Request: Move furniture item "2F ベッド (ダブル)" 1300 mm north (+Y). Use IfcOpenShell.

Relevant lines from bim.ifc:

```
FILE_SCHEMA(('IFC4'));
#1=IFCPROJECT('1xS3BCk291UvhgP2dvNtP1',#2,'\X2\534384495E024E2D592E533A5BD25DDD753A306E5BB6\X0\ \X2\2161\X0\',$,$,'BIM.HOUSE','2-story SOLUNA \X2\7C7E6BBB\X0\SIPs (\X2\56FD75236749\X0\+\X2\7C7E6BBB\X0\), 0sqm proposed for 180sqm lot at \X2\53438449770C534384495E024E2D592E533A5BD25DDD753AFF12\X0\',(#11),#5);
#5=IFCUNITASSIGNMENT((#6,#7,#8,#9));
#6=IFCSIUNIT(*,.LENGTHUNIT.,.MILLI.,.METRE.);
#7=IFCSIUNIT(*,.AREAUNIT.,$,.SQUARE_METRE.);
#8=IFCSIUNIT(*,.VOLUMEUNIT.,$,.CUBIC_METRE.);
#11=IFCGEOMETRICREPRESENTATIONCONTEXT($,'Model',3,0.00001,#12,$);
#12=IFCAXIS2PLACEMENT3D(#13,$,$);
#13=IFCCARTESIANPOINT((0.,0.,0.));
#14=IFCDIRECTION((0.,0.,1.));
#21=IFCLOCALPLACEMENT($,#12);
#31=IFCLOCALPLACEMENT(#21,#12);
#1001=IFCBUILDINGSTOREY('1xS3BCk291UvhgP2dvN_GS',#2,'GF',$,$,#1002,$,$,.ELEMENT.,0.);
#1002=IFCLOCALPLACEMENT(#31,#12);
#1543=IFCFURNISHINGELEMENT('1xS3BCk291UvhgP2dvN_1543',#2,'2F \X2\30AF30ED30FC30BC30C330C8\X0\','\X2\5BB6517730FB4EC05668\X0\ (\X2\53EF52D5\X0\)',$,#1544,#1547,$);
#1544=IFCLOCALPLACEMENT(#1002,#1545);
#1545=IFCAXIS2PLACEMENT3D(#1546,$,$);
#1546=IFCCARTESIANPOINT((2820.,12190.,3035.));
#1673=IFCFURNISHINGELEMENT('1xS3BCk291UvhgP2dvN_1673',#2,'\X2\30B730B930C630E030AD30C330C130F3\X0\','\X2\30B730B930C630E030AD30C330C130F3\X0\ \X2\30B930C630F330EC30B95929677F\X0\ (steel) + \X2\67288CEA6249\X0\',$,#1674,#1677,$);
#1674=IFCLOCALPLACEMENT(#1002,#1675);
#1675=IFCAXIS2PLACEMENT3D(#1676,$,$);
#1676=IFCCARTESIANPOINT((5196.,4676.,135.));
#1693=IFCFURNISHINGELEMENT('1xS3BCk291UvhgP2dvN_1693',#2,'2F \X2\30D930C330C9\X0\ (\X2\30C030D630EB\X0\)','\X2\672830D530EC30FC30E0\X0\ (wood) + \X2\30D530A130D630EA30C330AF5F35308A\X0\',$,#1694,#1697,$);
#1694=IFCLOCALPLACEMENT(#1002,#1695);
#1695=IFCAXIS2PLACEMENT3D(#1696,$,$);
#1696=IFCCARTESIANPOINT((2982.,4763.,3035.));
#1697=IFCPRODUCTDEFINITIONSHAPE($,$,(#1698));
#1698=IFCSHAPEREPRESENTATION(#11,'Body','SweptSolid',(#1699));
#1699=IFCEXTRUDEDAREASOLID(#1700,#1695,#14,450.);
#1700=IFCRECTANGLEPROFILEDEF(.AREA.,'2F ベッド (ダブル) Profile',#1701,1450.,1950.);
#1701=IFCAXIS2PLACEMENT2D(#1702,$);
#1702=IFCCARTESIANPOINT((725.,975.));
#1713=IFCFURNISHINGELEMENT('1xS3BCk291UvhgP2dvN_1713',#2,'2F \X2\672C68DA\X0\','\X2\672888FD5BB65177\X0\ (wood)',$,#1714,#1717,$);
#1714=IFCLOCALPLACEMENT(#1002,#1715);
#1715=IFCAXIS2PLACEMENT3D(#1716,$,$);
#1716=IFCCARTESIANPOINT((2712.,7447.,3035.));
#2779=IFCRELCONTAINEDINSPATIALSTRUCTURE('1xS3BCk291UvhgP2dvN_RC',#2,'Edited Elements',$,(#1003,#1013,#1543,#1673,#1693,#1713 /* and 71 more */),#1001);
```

```python
import ifcopenshell
import ifcopenshell.api.geometry
import ifcopenshell.util.placement
import ifcopenshell.util.unit

model = ifcopenshell.open("bim.ifc")
unit_scale = ifcopenshell.util.unit.calculate_unit_scale(model)

item = model.by_id(1693)
matrix = ifcopenshell.util.placement.get_local_placement(item.ObjectPlacement)
matrix[1, 3] += 1.3 / unit_scale
ifcopenshell.api.geometry.edit_object_placement(model, product=item, matrix=matrix, is_si=False)

print(ifcopenshell.util.placement.get_local_placement(item.ObjectPlacement).round(3) + 0.0)

model.write("bim_rev.ifc")
```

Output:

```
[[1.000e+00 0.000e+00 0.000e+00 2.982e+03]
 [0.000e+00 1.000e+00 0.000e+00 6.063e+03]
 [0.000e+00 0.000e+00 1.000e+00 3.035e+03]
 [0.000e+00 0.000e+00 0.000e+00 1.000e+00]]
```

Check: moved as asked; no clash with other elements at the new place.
